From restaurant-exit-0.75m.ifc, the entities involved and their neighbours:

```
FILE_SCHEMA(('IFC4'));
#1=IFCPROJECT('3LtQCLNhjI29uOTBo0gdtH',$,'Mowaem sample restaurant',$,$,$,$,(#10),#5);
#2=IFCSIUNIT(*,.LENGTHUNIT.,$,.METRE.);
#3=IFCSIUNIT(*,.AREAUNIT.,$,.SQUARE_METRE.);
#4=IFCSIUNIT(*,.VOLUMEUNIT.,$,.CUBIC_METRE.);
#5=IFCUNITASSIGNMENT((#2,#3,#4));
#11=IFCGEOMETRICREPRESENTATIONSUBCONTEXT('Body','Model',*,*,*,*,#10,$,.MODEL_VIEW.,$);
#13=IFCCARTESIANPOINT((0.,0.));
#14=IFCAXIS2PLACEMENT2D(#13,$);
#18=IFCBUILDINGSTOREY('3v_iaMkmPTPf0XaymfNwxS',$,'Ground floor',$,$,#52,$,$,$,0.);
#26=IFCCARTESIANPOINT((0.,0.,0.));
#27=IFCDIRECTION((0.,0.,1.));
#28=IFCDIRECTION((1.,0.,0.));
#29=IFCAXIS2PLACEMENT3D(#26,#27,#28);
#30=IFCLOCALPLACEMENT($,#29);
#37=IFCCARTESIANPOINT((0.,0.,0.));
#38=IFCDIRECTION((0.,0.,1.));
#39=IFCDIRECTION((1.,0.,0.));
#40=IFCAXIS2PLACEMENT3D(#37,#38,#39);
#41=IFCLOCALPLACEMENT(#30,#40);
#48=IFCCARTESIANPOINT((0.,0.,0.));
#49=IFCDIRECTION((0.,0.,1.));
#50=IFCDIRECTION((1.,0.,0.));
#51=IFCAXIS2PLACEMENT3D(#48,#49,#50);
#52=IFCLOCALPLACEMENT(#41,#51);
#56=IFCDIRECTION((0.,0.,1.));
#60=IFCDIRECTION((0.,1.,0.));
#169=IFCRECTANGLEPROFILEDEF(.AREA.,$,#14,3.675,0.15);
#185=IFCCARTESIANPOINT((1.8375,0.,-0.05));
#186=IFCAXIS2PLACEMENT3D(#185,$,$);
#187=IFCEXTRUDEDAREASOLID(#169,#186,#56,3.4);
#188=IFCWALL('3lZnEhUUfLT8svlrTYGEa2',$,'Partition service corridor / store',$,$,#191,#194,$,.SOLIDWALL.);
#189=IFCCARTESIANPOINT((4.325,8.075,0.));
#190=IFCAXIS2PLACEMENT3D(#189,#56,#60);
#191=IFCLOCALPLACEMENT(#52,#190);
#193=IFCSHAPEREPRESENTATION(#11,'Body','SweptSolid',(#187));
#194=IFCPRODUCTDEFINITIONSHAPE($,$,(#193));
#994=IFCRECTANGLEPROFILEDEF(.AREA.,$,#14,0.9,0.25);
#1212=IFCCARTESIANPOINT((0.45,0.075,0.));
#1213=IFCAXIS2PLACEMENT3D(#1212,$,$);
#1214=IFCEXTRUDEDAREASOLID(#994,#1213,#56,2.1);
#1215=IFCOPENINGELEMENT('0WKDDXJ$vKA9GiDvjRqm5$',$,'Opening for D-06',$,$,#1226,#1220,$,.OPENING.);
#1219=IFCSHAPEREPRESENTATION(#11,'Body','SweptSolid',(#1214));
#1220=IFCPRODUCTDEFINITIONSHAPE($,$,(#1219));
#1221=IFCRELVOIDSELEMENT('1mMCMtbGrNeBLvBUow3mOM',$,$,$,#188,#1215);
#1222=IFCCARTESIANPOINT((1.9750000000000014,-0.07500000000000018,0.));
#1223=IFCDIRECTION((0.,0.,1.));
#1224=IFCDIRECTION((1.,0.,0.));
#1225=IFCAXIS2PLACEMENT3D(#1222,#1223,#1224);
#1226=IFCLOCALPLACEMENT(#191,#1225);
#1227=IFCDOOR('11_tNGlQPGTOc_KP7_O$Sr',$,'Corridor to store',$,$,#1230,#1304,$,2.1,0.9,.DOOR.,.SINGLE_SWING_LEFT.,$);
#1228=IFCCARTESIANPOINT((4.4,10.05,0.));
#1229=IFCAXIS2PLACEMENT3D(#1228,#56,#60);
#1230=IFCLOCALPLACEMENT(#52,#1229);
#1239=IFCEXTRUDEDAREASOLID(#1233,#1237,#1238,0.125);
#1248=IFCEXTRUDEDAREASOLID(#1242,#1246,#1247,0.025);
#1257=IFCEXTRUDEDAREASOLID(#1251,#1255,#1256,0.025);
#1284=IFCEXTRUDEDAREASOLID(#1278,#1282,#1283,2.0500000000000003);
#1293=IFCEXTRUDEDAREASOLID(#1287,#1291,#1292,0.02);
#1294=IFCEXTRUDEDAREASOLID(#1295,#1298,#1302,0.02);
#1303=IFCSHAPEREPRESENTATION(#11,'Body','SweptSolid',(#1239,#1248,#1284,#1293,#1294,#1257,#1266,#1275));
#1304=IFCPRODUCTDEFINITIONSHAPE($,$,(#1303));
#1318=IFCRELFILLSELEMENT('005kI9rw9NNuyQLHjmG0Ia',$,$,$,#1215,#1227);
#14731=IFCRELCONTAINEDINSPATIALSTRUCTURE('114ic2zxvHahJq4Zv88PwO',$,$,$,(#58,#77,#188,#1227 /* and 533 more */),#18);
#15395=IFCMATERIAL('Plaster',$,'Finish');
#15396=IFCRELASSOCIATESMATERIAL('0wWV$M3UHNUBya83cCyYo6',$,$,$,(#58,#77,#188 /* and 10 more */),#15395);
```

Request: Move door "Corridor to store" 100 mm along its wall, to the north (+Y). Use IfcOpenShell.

```python
import ifcopenshell
import ifcopenshell.api.geometry
import ifcopenshell.util.placement
import ifcopenshell.util.unit

model = ifcopenshell.open("restaurant-exit-0.75m.ifc")
unit_scale = ifcopenshell.util.unit.calculate_unit_scale(model)

door = model.by_guid("11_tNGlQPGTOc_KP7_O$Sr")
opening = door.FillsVoids[0].RelatingOpeningElement
wall = opening.VoidsElements[0].RelatingBuildingElement

wall_matrix = ifcopenshell.util.placement.get_local_placement(wall.ObjectPlacement)
shift = wall_matrix[:3, 0] * 0.1 / unit_scale
before = ifcopenshell.util.placement.get_local_placement(door.ObjectPlacement)[:3, 3].copy()

# The door is not placed relative to its opening, so move both.
for product in (opening, door):
    matrix = ifcopenshell.util.placement.get_local_placement(product.ObjectPlacement)
    matrix[:3, 3] += shift
    ifcopenshell.api.geometry.edit_object_placement(model, product=product, matrix=matrix, is_si=False)

after = ifcopenshell.util.placement.get_local_placement(door.ObjectPlacement)[:3, 3]
print("door moved by", (after - before).round(3) + 0.0)

model.write("restaurant-exit-0.75m_updated.ifc")
```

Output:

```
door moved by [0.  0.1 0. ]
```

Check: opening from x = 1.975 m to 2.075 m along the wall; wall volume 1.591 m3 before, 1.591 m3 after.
